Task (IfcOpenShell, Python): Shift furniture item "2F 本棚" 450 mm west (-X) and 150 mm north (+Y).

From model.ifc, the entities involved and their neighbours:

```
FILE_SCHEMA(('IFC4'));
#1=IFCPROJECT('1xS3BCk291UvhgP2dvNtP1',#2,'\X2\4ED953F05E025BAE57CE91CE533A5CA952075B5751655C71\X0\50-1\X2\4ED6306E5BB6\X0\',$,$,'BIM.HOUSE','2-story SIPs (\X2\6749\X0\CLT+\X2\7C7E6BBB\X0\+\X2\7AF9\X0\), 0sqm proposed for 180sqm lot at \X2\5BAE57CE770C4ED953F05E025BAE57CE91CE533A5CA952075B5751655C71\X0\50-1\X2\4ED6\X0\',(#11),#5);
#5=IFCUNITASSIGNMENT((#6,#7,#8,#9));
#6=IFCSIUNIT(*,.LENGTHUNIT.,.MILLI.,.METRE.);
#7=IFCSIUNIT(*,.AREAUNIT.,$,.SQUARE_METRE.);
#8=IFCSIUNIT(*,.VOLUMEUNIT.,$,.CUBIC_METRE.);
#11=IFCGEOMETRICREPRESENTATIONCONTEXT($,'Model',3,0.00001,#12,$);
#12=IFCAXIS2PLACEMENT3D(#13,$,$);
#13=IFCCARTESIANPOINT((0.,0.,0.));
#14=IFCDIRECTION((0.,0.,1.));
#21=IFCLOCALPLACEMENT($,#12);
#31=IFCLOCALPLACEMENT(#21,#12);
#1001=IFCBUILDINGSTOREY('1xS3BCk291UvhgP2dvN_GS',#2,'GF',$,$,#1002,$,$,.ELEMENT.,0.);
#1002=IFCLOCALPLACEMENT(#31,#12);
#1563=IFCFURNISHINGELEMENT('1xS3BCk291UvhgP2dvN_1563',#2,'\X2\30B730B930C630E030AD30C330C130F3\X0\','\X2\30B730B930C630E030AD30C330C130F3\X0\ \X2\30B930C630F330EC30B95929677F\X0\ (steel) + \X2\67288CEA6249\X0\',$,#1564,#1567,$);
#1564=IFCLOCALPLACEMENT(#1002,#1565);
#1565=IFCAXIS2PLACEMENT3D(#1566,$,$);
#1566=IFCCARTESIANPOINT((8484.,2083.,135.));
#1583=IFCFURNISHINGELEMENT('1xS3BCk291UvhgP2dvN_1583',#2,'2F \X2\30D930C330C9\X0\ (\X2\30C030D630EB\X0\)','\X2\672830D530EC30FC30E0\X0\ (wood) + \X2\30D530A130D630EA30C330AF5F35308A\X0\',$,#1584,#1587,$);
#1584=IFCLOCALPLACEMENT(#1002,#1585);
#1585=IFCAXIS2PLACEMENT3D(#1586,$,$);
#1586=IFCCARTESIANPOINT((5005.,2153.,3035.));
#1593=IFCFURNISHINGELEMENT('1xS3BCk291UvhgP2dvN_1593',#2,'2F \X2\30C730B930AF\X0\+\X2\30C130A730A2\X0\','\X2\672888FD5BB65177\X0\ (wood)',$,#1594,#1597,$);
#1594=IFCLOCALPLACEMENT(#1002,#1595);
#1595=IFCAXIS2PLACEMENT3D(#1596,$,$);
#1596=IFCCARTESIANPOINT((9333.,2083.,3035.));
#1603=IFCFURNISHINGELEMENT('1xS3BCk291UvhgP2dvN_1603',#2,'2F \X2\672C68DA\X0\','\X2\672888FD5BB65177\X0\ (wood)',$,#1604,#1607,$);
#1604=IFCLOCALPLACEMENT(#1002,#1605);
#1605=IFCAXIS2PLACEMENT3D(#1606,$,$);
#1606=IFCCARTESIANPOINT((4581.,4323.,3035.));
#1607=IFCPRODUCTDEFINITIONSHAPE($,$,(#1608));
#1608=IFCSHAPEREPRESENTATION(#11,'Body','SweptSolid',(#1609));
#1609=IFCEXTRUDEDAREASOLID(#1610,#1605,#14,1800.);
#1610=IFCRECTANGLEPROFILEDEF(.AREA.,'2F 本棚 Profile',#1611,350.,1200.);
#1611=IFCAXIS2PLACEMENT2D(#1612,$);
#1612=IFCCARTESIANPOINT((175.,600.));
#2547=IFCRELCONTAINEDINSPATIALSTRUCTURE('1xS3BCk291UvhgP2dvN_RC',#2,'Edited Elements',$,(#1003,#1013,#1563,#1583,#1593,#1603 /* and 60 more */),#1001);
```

```python
import ifcopenshell
import ifcopenshell.api.geometry
import ifcopenshell.util.placement
import ifcopenshell.util.unit

model = ifcopenshell.open("model.ifc")
unit_scale = ifcopenshell.util.unit.calculate_unit_scale(model)

item = model.by_guid("1xS3BCk291UvhgP2dvN_1603")
matrix = ifcopenshell.util.placement.get_local_placement(item.ObjectPlacement)
matrix[0, 3] -= 0.45 / unit_scale
matrix[1, 3] += 0.15 / unit_scale
ifcopenshell.api.geometry.edit_object_placement(model, product=item, matrix=matrix, is_si=False)

print(ifcopenshell.util.placement.get_local_placement(item.ObjectPlacement).round(3) + 0.0)

model.write("model_v2.ifc")
```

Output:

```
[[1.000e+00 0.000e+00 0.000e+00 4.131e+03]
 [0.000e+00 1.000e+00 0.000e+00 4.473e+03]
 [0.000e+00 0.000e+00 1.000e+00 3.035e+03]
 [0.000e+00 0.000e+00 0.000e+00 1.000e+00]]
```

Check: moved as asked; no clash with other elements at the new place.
